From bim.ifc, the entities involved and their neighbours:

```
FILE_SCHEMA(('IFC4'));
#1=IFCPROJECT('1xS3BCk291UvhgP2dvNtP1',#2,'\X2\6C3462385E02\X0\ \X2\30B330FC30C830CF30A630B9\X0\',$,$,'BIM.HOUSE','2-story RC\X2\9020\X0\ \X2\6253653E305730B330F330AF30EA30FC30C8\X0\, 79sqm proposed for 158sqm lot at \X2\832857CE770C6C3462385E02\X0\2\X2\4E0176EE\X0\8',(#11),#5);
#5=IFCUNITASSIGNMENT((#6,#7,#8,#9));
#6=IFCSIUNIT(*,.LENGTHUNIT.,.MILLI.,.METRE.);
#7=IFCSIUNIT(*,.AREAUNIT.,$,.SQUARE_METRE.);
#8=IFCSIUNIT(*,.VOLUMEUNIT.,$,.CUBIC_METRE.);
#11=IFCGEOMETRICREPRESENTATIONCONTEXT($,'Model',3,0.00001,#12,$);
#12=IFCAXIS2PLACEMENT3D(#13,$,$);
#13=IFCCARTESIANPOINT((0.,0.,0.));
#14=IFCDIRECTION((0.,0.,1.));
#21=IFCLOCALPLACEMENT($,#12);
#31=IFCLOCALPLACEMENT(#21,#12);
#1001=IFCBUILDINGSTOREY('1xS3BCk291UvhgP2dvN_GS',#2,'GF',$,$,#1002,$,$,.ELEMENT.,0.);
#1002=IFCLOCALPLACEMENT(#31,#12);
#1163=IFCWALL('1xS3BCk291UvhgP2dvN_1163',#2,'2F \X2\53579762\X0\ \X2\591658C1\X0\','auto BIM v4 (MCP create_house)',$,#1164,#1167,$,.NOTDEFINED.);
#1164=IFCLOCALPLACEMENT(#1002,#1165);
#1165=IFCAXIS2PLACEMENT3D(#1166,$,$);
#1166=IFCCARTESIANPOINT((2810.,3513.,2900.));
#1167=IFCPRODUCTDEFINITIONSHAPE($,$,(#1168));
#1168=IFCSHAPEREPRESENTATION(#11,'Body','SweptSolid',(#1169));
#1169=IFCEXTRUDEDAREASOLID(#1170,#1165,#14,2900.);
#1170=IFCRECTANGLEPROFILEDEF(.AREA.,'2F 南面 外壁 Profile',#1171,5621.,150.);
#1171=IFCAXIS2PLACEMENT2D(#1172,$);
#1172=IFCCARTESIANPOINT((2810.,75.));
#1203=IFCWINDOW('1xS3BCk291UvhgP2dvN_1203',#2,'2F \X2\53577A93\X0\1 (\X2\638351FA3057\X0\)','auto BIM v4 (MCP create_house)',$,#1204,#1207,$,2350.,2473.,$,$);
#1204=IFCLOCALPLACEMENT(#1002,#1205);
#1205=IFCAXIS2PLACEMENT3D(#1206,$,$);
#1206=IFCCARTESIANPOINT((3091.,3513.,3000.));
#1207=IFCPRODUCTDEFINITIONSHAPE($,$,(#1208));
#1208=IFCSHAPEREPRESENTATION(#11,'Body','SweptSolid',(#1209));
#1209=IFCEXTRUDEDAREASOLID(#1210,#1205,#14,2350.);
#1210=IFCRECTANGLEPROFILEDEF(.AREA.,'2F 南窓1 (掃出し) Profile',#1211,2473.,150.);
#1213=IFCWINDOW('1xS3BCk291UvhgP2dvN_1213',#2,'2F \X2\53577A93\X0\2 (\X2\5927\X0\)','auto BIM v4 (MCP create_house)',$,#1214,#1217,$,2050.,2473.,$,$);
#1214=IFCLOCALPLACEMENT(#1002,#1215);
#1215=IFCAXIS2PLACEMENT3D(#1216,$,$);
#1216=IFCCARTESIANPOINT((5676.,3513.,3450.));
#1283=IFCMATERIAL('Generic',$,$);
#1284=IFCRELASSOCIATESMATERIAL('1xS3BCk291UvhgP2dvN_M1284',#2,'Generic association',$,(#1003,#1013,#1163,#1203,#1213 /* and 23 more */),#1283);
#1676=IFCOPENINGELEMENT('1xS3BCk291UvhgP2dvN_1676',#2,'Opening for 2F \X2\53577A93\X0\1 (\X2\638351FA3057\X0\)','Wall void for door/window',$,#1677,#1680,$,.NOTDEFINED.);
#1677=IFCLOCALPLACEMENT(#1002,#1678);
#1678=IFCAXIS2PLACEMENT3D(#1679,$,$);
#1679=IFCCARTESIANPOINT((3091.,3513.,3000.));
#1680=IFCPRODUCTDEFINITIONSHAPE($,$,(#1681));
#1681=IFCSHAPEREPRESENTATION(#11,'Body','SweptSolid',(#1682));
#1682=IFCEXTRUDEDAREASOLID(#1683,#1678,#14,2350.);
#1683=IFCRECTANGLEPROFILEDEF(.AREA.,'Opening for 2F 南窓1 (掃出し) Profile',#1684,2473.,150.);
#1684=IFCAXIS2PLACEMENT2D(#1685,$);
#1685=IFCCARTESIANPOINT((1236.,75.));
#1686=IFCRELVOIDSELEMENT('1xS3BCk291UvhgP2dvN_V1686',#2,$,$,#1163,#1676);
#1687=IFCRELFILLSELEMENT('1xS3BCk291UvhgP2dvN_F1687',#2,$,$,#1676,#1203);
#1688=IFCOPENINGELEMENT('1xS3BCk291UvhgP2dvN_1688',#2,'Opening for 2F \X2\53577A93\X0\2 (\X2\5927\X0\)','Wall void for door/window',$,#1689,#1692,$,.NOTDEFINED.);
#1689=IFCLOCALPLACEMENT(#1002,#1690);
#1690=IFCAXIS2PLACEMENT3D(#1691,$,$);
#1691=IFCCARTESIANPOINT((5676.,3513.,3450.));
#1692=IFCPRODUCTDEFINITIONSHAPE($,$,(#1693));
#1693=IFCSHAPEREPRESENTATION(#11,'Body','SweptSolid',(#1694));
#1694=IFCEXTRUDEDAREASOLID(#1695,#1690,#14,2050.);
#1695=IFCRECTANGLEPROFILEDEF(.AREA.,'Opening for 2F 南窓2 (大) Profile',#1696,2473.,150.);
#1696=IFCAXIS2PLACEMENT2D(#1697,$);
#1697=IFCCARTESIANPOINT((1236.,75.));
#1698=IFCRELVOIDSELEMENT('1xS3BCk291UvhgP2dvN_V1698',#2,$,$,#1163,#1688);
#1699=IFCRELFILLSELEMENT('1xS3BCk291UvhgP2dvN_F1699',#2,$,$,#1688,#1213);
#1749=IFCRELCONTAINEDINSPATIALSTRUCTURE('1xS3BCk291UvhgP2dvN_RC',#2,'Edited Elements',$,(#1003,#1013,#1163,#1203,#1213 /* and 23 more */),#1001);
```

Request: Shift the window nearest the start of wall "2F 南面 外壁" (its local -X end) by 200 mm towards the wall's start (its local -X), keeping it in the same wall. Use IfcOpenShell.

```python
import ifcopenshell
import ifcopenshell.api.geometry
import ifcopenshell.util.placement
import ifcopenshell.util.unit

model = ifcopenshell.open("bim.ifc")
unit_scale = ifcopenshell.util.unit.calculate_unit_scale(model)

window = model.by_guid("1xS3BCk291UvhgP2dvN_1203")
opening = window.FillsVoids[0].RelatingOpeningElement
wall = opening.VoidsElements[0].RelatingBuildingElement

wall_matrix = ifcopenshell.util.placement.get_local_placement(wall.ObjectPlacement)
shift = wall_matrix[:3, 0] * -0.2 / unit_scale
before = ifcopenshell.util.placement.get_local_placement(window.ObjectPlacement)[:3, 3].copy()

# The window is not placed relative to its opening, so move both.
for product in (opening, window):
    matrix = ifcopenshell.util.placement.get_local_placement(product.ObjectPlacement)
    matrix[:3, 3] += shift
    ifcopenshell.api.geometry.edit_object_placement(model, product=product, matrix=matrix, is_si=False)

after = ifcopenshell.util.placement.get_local_placement(window.ObjectPlacement)[:3, 3]
print("window moved by", (after - before).round(3) + 0.0)

model.write("bim_edited.ifc")
```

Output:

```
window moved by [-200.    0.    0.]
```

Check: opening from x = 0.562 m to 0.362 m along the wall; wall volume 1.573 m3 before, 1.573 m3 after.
